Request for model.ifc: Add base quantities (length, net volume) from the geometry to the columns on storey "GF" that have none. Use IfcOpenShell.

First a look at what the model holds.

```python
import ifcopenshell
import ifcopenshell.util.element
import ifcopenshell.util.unit

model = ifcopenshell.open("model.ifc")
print(model.schema)
for unit_type in ("LENGTHUNIT", "AREAUNIT", "VOLUMEUNIT"):
    print(unit_type, ifcopenshell.util.unit.calculate_unit_scale(model, unit_type))
storey = next(s for s in model.by_type("IfcBuildingStorey") if s.Name == "GF")
columns = [e for e in ifcopenshell.util.element.get_decomposition(storey) if e.is_a("IfcColumn")]
for e in sorted(columns, key=lambda e: e.id()):
    print(e.id(), e.is_a(), e.Name, list(ifcopenshell.util.element.get_psets(e, qtos_only=True)), sep=" | ")
```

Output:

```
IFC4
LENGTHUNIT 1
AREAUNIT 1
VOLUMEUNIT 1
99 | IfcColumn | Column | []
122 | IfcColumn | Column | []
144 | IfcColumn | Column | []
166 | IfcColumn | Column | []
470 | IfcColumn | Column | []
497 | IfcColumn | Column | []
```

```python
import ifcopenshell
import ifcopenshell.api.pset
import ifcopenshell.geom
import ifcopenshell.util.element
import ifcopenshell.util.shape
import ifcopenshell.util.unit

model = ifcopenshell.open("model.ifc")
unit_scale = ifcopenshell.util.unit.calculate_unit_scale(model)
volume_scale = ifcopenshell.util.unit.calculate_unit_scale(model, "VOLUMEUNIT")
settings = ifcopenshell.geom.settings()

storey = next(s for s in model.by_type("IfcBuildingStorey") if s.Name == "GF")
columns = [e for e in ifcopenshell.util.element.get_decomposition(storey) if e.is_a("IfcColumn")]

for e in sorted(columns, key=lambda e: e.id()):
    if ifcopenshell.util.element.get_psets(e, qtos_only=True, should_inherit=False):
        continue
    # Geometry comes back in metres, in the element's own axes.
    shape = ifcopenshell.geom.create_shape(settings, e)
    values = {
        "Length": ifcopenshell.util.shape.get_z(shape.geometry) / unit_scale,
        "NetVolume": ifcopenshell.util.shape.get_volume(shape.geometry) / volume_scale,
    }
    qto = ifcopenshell.api.pset.add_qto(model, product=e, name="Qto_ColumnBaseQuantities")
    ifcopenshell.api.pset.edit_qto(model, qto=qto, properties=values)
    print(e.id(), {k: round(v, 3) for k, v in values.items()})

model.write("model_v2.ifc")
```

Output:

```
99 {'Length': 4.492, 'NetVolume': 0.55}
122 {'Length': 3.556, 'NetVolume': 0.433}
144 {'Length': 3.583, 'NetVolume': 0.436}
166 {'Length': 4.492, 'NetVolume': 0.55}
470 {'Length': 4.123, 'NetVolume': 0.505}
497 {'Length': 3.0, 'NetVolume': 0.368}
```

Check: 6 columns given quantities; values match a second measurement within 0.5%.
